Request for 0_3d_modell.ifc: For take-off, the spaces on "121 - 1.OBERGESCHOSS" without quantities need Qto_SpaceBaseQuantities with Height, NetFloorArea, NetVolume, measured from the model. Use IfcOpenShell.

First a look at what the model holds.

```python
import ifcopenshell
import ifcopenshell.util.element
import ifcopenshell.util.unit

model = ifcopenshell.open("0_3d_modell.ifc")
print(model.schema)
for unit_type in ("LENGTHUNIT", "AREAUNIT", "VOLUMEUNIT"):
    print(unit_type, ifcopenshell.util.unit.calculate_unit_scale(model, unit_type))
storey = next(s for s in model.by_type("IfcBuildingStorey") if s.Name == "121 - 1.OBERGESCHOSS")
spaces = [e for e in ifcopenshell.util.element.get_decomposition(storey) if e.is_a("IfcSpace")]
for e in sorted(spaces, key=lambda e: e.id()):
    print(e.id(), e.is_a(), e.Name, list(ifcopenshell.util.element.get_psets(e, qtos_only=True)), sep=" | ")
```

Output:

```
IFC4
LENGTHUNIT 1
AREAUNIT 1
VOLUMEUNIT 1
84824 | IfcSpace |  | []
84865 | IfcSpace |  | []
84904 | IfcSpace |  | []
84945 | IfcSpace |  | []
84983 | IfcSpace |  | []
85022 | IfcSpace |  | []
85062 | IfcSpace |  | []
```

```python
import ifcopenshell
import ifcopenshell.api.pset
import ifcopenshell.geom
import ifcopenshell.util.element
import ifcopenshell.util.shape
import ifcopenshell.util.unit

model = ifcopenshell.open("0_3d_modell.ifc")
unit_scale = ifcopenshell.util.unit.calculate_unit_scale(model)
area_scale = ifcopenshell.util.unit.calculate_unit_scale(model, "AREAUNIT")
volume_scale = ifcopenshell.util.unit.calculate_unit_scale(model, "VOLUMEUNIT")
settings = ifcopenshell.geom.settings()

storey = next(s for s in model.by_type("IfcBuildingStorey") if s.Name == "121 - 1.OBERGESCHOSS")
spaces = [e for e in ifcopenshell.util.element.get_decomposition(storey) if e.is_a("IfcSpace")]

for e in sorted(spaces, key=lambda e: e.id()):
    if ifcopenshell.util.element.get_psets(e, qtos_only=True, should_inherit=False):
        continue
    # Geometry comes back in metres, in the element's own axes.
    shape = ifcopenshell.geom.create_shape(settings, e)
    values = {
        "Height": ifcopenshell.util.shape.get_z(shape.geometry) / unit_scale,
        "NetFloorArea": ifcopenshell.util.shape.get_footprint_area(shape.geometry) / area_scale,
        "NetVolume": ifcopenshell.util.shape.get_volume(shape.geometry) / volume_scale,
    }
    qto = ifcopenshell.api.pset.add_qto(model, product=e, name="Qto_SpaceBaseQuantities")
    ifcopenshell.api.pset.edit_qto(model, qto=qto, properties=values)
    print(e.id(), {k: round(v, 3) for k, v in values.items()})

model.write("0_3d_modell_rev.ifc")
```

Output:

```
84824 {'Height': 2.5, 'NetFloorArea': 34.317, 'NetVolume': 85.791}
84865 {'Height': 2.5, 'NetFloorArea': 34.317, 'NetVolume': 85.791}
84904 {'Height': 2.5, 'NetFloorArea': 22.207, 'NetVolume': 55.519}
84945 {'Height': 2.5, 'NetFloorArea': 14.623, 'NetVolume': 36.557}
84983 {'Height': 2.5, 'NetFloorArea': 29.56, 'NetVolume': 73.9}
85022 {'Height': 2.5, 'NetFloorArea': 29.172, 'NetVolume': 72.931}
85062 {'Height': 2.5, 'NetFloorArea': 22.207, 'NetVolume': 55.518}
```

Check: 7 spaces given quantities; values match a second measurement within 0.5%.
